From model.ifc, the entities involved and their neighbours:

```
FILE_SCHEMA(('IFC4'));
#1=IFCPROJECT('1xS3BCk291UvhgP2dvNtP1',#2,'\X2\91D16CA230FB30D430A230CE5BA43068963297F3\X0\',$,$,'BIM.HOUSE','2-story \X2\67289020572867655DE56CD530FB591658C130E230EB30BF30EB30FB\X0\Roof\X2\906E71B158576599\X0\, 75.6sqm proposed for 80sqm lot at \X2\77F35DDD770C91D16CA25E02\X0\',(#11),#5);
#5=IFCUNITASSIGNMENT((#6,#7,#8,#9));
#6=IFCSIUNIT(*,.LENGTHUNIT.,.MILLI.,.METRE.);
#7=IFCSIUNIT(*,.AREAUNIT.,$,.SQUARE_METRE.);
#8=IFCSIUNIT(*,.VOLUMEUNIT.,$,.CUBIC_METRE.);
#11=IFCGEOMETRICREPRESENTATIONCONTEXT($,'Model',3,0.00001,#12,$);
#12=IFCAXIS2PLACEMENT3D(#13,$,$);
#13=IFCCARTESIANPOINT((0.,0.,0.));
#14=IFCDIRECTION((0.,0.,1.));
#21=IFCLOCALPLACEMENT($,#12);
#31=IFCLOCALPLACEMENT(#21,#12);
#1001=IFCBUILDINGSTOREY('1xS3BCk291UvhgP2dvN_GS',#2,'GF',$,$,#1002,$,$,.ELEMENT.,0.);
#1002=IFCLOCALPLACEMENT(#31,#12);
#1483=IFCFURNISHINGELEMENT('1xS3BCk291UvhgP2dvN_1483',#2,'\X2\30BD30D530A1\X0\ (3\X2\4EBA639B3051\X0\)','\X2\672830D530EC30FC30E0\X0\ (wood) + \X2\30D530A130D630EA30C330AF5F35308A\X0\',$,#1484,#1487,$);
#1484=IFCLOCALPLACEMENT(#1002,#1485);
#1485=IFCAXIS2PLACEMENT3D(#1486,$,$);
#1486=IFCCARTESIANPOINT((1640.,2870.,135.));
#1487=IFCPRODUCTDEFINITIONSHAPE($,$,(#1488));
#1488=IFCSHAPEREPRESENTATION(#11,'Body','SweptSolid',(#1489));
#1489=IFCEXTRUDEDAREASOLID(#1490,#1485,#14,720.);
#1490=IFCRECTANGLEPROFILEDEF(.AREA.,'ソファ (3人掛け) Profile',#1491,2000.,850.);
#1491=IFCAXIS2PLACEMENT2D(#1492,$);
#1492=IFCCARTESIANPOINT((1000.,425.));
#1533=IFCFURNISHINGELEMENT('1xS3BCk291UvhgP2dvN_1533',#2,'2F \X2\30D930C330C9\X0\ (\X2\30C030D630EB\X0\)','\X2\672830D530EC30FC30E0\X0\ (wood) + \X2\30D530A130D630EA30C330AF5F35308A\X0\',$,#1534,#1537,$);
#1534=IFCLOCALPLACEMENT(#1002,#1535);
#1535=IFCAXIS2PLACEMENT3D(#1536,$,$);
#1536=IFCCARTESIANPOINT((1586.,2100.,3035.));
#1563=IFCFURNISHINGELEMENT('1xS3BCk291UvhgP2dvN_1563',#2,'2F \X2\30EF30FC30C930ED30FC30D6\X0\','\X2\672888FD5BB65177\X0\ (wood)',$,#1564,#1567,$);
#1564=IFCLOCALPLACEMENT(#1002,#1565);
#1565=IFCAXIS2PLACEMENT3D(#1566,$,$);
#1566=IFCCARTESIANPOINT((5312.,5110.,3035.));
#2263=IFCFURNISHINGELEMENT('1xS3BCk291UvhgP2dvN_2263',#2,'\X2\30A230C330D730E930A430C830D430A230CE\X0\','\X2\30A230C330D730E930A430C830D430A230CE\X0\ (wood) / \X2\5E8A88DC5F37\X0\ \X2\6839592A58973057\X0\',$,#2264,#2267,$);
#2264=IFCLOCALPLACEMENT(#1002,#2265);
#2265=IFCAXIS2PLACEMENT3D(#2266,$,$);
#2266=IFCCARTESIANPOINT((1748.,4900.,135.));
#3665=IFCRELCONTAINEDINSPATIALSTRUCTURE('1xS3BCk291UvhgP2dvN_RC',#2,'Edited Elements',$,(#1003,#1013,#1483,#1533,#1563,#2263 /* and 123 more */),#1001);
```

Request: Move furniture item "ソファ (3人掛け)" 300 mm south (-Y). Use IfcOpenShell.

```python
import ifcopenshell
import ifcopenshell.api.geometry
import ifcopenshell.util.placement
import ifcopenshell.util.unit

model = ifcopenshell.open("model.ifc")
unit_scale = ifcopenshell.util.unit.calculate_unit_scale(model)

item = model.by_guid("1xS3BCk291UvhgP2dvN_1483")
matrix = ifcopenshell.util.placement.get_local_placement(item.ObjectPlacement)
matrix[1, 3] -= 0.3 / unit_scale
ifcopenshell.api.geometry.edit_object_placement(model, product=item, matrix=matrix, is_si=False)

print(ifcopenshell.util.placement.get_local_placement(item.ObjectPlacement).round(3) + 0.0)

model.write("model_rev.ifc")
```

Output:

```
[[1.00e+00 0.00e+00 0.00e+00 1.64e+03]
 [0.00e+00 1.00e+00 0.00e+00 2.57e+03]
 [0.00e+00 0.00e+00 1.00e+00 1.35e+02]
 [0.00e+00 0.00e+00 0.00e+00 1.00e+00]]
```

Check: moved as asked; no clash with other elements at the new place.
